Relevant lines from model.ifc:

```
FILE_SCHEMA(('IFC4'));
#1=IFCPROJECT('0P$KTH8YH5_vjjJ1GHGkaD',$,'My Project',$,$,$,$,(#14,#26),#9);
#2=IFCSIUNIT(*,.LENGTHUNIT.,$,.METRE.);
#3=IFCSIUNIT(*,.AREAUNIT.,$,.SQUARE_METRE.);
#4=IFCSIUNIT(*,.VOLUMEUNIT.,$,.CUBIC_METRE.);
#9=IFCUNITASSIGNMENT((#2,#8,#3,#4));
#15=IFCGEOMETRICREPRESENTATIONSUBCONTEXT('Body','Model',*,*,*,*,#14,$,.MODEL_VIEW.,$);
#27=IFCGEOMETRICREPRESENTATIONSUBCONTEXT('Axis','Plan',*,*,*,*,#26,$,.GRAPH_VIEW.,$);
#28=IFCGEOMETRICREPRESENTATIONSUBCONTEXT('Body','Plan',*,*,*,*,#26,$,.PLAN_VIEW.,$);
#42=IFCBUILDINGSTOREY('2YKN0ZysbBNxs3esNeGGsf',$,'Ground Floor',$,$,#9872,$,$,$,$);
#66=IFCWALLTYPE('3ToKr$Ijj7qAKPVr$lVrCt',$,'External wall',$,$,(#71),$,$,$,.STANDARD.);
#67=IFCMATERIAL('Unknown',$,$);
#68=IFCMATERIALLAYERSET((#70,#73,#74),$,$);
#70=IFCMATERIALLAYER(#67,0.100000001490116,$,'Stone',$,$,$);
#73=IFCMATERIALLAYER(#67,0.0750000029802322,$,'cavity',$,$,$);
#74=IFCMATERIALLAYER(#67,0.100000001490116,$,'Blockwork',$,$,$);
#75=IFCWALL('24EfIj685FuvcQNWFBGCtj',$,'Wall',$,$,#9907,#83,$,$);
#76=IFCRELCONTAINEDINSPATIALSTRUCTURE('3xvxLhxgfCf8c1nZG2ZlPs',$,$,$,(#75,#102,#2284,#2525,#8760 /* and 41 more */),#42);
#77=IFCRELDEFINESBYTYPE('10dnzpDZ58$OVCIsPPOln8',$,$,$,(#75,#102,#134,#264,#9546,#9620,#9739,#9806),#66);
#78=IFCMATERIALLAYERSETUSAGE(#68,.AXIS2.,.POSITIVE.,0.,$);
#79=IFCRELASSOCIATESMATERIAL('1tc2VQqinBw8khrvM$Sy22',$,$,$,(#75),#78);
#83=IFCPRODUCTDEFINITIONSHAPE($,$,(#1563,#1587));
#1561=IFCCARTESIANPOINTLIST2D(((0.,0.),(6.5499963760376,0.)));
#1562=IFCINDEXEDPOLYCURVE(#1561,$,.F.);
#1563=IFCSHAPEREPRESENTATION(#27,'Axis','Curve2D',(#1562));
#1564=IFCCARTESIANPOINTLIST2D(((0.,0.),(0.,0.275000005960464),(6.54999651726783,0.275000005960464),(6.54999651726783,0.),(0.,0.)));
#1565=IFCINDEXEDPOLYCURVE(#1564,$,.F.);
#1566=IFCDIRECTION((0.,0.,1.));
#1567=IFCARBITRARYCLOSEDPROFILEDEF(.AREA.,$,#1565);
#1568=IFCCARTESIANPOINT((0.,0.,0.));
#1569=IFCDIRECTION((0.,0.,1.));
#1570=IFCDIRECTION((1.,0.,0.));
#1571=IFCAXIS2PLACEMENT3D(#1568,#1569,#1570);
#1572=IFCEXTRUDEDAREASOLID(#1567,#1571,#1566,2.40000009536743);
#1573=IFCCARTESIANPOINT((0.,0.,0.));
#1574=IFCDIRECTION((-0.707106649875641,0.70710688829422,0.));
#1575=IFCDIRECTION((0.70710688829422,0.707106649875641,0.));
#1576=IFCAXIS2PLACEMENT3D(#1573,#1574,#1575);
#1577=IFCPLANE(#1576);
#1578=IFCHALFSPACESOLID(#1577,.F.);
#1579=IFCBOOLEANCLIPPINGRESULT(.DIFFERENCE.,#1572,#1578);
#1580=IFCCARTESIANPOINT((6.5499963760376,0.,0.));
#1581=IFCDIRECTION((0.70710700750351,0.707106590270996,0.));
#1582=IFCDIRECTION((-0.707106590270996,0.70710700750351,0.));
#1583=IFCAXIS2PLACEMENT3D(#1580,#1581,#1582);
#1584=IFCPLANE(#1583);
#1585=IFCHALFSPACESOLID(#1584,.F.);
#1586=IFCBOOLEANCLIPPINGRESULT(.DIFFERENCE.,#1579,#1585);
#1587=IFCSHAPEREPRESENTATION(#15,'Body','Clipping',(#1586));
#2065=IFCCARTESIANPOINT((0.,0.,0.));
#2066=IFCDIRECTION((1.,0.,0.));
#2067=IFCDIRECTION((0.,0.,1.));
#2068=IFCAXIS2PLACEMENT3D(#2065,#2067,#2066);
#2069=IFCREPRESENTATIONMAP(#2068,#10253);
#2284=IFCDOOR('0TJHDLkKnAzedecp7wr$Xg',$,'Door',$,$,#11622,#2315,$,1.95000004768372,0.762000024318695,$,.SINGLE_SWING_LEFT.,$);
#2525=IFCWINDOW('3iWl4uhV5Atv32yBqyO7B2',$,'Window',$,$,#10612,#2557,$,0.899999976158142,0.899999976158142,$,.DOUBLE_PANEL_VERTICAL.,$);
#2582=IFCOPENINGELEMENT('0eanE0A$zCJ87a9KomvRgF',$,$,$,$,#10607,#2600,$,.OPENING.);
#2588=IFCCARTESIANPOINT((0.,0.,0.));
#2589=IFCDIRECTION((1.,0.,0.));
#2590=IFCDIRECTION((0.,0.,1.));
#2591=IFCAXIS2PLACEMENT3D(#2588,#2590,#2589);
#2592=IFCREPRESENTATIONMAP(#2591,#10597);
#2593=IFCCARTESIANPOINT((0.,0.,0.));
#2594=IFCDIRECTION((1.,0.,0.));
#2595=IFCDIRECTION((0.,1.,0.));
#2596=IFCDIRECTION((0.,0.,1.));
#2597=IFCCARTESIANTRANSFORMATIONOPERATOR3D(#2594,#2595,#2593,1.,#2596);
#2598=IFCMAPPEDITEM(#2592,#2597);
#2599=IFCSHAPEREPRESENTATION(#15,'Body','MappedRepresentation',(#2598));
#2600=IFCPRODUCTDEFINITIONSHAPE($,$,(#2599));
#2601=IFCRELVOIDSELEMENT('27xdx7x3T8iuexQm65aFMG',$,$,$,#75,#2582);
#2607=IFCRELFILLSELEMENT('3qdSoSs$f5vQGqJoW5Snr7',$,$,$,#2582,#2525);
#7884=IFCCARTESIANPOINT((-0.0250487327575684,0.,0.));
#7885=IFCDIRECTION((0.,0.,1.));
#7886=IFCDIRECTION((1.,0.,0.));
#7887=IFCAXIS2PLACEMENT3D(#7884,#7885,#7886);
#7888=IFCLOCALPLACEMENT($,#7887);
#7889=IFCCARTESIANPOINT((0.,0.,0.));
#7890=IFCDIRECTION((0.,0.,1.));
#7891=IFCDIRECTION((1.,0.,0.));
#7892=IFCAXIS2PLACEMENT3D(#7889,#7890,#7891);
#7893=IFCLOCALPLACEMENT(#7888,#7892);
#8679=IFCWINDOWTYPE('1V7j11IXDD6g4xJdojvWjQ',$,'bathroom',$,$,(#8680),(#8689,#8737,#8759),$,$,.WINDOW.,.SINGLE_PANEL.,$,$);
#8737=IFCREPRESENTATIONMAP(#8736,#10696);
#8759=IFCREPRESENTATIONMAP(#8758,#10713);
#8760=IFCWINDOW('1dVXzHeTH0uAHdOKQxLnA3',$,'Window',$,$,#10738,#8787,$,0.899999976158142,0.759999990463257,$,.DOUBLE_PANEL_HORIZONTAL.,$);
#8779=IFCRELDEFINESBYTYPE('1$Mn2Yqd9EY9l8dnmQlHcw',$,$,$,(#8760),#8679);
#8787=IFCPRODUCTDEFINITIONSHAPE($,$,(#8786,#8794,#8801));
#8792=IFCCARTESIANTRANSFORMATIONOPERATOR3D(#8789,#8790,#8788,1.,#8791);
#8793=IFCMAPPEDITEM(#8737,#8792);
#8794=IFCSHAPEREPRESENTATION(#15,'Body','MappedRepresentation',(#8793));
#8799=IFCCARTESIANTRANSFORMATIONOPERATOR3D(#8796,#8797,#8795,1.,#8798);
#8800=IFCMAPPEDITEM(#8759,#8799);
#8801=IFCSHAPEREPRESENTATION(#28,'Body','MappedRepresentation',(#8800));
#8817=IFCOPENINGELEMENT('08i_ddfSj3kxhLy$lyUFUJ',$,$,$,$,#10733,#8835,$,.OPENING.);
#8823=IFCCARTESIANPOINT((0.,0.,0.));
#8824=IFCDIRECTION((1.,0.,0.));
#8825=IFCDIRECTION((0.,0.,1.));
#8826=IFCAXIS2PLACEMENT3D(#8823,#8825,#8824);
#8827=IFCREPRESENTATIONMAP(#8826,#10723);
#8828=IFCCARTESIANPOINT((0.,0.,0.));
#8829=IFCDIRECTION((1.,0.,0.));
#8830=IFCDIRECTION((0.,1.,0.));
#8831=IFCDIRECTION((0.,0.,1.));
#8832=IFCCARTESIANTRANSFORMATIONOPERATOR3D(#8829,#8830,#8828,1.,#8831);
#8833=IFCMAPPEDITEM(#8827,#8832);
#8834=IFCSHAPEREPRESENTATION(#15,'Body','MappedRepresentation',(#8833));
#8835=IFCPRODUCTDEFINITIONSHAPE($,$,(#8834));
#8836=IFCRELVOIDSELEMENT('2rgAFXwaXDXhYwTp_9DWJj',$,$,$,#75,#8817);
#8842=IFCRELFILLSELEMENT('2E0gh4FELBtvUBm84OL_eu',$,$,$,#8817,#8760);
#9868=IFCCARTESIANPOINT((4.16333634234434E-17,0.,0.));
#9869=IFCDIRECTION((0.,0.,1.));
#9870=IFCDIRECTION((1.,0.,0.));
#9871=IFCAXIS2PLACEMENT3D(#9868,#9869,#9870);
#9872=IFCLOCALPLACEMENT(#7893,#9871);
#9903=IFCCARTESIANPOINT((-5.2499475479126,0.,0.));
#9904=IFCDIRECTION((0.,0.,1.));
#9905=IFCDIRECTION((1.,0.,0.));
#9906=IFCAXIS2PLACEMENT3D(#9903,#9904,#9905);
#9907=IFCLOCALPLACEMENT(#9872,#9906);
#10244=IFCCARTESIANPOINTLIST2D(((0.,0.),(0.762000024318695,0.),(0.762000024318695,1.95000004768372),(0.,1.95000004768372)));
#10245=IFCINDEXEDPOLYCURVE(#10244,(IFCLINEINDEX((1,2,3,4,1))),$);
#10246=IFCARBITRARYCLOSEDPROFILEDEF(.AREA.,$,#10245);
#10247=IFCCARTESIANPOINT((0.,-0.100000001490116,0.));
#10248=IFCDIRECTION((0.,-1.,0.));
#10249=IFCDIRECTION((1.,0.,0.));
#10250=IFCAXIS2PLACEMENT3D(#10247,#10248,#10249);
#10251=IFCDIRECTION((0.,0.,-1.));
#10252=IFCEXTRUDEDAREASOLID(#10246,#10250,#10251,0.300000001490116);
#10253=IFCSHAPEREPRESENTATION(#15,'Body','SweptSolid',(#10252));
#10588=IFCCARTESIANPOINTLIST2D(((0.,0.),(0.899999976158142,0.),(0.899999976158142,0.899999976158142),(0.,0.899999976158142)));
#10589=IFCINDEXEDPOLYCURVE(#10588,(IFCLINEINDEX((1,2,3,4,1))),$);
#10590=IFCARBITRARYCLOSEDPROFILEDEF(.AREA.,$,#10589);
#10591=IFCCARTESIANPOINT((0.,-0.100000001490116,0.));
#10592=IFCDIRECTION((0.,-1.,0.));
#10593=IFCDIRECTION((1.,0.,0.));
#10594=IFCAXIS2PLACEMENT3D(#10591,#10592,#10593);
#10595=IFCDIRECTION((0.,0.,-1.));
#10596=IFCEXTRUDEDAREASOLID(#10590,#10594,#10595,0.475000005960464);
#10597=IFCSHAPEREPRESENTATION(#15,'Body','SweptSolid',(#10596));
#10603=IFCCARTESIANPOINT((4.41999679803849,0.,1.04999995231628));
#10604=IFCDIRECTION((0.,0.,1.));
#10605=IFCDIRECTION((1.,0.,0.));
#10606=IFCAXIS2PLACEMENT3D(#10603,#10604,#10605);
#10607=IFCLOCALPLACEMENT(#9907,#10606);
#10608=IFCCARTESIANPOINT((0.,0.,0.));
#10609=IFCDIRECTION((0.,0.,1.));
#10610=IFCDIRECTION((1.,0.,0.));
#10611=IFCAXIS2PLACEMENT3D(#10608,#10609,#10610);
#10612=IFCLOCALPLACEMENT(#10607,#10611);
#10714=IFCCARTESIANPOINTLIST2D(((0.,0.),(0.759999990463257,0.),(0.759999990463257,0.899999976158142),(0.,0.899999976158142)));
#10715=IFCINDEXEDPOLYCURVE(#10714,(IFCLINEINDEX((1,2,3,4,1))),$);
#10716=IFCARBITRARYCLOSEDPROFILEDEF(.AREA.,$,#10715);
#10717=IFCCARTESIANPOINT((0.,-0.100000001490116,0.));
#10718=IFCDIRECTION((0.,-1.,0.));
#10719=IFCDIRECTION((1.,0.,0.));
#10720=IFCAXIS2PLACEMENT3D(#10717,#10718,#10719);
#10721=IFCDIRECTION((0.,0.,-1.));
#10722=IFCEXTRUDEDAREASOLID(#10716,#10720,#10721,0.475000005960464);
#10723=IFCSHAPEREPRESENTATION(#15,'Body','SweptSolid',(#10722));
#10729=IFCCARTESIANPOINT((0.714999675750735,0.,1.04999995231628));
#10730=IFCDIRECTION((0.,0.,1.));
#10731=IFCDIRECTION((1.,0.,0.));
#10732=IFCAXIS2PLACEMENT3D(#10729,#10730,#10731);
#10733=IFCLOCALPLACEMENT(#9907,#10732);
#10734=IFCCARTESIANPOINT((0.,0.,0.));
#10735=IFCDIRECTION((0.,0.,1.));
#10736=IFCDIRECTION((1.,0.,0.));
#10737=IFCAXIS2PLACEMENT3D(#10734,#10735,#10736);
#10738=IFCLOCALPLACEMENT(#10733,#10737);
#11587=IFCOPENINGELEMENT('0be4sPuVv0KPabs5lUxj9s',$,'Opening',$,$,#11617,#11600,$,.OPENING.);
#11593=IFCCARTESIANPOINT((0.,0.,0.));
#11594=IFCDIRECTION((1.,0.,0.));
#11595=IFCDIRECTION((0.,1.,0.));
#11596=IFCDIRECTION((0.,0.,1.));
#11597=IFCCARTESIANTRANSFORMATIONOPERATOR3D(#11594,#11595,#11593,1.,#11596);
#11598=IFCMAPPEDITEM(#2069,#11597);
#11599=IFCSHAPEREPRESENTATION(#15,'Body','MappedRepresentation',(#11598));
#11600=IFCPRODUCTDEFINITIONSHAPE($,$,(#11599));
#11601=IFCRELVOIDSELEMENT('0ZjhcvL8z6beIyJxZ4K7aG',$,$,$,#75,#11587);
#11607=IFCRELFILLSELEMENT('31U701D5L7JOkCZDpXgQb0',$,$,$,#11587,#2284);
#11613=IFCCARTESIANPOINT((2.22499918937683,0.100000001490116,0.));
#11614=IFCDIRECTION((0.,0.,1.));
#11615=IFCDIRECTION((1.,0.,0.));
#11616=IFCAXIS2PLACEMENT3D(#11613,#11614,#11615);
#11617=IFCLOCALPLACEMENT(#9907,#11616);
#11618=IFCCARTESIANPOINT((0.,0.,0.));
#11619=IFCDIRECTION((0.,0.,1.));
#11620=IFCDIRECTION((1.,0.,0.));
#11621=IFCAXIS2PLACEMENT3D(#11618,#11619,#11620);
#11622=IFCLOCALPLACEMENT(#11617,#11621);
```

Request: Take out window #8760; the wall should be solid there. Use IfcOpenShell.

```python
import ifcopenshell
import ifcopenshell.api.feature
import ifcopenshell.api.root
import ifcopenshell.geom
import ifcopenshell.util.shape

model = ifcopenshell.open("model.ifc")
settings = ifcopenshell.geom.settings()


def volume(element):
    """Net volume in cubic metres, openings subtracted."""
    shape = ifcopenshell.geom.create_shape(settings, element)
    return ifcopenshell.util.shape.get_volume(shape.geometry)


window = model.by_id(8760)
opening = window.FillsVoids[0].RelatingOpeningElement
wall = opening.VoidsElements[0].RelatingBuildingElement
before = volume(wall)

ifcopenshell.api.root.remove_product(model, product=window)
ifcopenshell.api.feature.remove_feature(model, feature=opening)

after = volume(wall)

print(f"wall volume {before:.3f} -> {after:.3f} m3")

model.write("model_v2.ifc")
```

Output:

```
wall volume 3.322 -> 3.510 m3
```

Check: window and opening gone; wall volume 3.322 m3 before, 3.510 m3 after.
